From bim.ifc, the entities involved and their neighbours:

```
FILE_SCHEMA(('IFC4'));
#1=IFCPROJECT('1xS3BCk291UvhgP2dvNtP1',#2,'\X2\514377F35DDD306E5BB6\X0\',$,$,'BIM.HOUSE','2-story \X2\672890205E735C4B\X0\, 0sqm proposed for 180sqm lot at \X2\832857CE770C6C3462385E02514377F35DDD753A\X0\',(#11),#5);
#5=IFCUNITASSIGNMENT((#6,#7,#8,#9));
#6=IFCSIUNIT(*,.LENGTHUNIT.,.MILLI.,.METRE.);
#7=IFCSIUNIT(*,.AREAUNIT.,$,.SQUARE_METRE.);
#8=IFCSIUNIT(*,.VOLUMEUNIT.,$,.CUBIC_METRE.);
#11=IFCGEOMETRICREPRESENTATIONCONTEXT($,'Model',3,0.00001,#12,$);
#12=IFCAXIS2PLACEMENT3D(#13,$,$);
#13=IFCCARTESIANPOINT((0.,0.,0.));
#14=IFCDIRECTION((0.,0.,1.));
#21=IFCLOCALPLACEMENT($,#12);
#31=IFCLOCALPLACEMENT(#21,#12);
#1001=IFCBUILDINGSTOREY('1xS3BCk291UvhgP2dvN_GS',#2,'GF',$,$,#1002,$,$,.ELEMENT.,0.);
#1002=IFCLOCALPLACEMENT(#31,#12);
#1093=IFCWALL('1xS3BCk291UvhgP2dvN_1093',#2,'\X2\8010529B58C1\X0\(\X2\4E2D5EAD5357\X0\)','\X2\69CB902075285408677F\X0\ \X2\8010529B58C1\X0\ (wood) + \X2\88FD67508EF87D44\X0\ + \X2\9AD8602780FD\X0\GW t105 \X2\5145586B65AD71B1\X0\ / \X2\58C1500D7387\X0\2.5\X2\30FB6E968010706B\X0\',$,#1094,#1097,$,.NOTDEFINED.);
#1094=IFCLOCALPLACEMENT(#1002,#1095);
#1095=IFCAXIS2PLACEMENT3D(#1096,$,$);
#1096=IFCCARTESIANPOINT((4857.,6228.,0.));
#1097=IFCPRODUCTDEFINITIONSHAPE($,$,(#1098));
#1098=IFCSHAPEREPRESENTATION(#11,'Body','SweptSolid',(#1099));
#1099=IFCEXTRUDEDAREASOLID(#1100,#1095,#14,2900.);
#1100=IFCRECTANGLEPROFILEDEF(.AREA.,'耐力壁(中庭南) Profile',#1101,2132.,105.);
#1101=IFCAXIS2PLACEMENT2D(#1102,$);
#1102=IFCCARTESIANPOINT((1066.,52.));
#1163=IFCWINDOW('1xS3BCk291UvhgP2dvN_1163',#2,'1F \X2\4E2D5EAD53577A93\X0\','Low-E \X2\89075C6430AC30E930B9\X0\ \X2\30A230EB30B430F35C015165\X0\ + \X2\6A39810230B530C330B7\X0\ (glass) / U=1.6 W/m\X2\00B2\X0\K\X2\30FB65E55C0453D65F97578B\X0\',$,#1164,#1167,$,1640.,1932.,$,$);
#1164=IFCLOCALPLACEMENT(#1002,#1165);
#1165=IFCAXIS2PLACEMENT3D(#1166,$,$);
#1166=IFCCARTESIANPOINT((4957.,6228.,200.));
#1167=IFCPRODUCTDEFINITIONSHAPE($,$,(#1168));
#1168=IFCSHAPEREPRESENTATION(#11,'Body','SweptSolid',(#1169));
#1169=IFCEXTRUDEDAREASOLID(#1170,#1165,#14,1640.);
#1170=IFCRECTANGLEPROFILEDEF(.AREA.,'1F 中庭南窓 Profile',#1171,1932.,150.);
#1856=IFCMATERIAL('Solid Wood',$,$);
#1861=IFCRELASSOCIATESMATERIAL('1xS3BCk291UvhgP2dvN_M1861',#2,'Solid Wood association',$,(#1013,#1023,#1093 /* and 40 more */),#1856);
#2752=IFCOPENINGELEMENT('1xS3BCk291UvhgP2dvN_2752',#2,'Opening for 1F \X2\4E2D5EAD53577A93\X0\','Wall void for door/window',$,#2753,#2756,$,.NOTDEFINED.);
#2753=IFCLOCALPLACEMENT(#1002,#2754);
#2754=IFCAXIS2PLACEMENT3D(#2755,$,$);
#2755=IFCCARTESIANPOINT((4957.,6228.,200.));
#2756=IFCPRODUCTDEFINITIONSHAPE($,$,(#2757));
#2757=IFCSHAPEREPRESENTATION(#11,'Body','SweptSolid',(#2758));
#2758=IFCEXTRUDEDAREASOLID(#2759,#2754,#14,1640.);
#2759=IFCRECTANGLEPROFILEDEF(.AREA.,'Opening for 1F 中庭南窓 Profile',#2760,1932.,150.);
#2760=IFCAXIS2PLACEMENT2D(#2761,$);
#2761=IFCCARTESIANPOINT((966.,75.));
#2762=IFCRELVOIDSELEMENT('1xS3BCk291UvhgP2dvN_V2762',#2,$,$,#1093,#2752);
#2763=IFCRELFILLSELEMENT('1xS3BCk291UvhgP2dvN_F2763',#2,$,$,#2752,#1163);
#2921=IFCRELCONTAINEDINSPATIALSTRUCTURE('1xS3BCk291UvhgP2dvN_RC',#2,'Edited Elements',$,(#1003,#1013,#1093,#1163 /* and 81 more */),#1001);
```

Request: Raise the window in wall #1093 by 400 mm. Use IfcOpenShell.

```python
import numpy as np
import ifcopenshell
import ifcopenshell.api.geometry
import ifcopenshell.util.placement
import ifcopenshell.util.unit

model = ifcopenshell.open("bim.ifc")
unit_scale = ifcopenshell.util.unit.calculate_unit_scale(model)

window = model.by_id(1163)
opening = window.FillsVoids[0].RelatingOpeningElement
dz = 0.4 / unit_scale

shift = np.array([0.0, 0.0, dz])
# The window is not placed relative to its opening, so move both.
for product in (opening, window):
    matrix = ifcopenshell.util.placement.get_local_placement(product.ObjectPlacement)
    matrix[:3, 3] += shift
    ifcopenshell.api.geometry.edit_object_placement(model, product=product, matrix=matrix, is_si=False)

print(f"moved by {dz * unit_scale:+.3f} m")

model.write("bim_rev.ifc")
```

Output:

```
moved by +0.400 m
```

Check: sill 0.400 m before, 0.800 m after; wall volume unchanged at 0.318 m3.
